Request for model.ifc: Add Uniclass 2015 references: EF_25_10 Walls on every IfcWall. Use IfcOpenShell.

First a look at what the model holds.

```python
import ifcopenshell

model = ifcopenshell.open("model.ifc")
print(model.schema)
print("classifications:", [c.Name for c in model.by_type("IfcClassification")])
for ifc_class in ("IfcDoor", "IfcRoof", "IfcStair", "IfcWall", "IfcWindow"):
    print(ifc_class, len(model.by_type(ifc_class)))
```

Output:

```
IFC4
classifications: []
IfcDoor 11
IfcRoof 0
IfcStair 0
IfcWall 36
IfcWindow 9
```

```python
import ifcopenshell
import ifcopenshell.api.classification

model = ifcopenshell.open("model.ifc")

system = ifcopenshell.api.classification.add_classification(model, classification="Uniclass 2015")

codes = {
    "IfcWall": ("EF_25_10", "Walls"),
}
for ifc_class, (code, name) in codes.items():
    products = model.by_type(ifc_class)
    ifcopenshell.api.classification.add_reference(
        model, products=products, classification=system, identification=code, name=name
    )
    print(code, len(products))

model.write("model_rev.ifc")
```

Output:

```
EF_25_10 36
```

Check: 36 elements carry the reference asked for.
